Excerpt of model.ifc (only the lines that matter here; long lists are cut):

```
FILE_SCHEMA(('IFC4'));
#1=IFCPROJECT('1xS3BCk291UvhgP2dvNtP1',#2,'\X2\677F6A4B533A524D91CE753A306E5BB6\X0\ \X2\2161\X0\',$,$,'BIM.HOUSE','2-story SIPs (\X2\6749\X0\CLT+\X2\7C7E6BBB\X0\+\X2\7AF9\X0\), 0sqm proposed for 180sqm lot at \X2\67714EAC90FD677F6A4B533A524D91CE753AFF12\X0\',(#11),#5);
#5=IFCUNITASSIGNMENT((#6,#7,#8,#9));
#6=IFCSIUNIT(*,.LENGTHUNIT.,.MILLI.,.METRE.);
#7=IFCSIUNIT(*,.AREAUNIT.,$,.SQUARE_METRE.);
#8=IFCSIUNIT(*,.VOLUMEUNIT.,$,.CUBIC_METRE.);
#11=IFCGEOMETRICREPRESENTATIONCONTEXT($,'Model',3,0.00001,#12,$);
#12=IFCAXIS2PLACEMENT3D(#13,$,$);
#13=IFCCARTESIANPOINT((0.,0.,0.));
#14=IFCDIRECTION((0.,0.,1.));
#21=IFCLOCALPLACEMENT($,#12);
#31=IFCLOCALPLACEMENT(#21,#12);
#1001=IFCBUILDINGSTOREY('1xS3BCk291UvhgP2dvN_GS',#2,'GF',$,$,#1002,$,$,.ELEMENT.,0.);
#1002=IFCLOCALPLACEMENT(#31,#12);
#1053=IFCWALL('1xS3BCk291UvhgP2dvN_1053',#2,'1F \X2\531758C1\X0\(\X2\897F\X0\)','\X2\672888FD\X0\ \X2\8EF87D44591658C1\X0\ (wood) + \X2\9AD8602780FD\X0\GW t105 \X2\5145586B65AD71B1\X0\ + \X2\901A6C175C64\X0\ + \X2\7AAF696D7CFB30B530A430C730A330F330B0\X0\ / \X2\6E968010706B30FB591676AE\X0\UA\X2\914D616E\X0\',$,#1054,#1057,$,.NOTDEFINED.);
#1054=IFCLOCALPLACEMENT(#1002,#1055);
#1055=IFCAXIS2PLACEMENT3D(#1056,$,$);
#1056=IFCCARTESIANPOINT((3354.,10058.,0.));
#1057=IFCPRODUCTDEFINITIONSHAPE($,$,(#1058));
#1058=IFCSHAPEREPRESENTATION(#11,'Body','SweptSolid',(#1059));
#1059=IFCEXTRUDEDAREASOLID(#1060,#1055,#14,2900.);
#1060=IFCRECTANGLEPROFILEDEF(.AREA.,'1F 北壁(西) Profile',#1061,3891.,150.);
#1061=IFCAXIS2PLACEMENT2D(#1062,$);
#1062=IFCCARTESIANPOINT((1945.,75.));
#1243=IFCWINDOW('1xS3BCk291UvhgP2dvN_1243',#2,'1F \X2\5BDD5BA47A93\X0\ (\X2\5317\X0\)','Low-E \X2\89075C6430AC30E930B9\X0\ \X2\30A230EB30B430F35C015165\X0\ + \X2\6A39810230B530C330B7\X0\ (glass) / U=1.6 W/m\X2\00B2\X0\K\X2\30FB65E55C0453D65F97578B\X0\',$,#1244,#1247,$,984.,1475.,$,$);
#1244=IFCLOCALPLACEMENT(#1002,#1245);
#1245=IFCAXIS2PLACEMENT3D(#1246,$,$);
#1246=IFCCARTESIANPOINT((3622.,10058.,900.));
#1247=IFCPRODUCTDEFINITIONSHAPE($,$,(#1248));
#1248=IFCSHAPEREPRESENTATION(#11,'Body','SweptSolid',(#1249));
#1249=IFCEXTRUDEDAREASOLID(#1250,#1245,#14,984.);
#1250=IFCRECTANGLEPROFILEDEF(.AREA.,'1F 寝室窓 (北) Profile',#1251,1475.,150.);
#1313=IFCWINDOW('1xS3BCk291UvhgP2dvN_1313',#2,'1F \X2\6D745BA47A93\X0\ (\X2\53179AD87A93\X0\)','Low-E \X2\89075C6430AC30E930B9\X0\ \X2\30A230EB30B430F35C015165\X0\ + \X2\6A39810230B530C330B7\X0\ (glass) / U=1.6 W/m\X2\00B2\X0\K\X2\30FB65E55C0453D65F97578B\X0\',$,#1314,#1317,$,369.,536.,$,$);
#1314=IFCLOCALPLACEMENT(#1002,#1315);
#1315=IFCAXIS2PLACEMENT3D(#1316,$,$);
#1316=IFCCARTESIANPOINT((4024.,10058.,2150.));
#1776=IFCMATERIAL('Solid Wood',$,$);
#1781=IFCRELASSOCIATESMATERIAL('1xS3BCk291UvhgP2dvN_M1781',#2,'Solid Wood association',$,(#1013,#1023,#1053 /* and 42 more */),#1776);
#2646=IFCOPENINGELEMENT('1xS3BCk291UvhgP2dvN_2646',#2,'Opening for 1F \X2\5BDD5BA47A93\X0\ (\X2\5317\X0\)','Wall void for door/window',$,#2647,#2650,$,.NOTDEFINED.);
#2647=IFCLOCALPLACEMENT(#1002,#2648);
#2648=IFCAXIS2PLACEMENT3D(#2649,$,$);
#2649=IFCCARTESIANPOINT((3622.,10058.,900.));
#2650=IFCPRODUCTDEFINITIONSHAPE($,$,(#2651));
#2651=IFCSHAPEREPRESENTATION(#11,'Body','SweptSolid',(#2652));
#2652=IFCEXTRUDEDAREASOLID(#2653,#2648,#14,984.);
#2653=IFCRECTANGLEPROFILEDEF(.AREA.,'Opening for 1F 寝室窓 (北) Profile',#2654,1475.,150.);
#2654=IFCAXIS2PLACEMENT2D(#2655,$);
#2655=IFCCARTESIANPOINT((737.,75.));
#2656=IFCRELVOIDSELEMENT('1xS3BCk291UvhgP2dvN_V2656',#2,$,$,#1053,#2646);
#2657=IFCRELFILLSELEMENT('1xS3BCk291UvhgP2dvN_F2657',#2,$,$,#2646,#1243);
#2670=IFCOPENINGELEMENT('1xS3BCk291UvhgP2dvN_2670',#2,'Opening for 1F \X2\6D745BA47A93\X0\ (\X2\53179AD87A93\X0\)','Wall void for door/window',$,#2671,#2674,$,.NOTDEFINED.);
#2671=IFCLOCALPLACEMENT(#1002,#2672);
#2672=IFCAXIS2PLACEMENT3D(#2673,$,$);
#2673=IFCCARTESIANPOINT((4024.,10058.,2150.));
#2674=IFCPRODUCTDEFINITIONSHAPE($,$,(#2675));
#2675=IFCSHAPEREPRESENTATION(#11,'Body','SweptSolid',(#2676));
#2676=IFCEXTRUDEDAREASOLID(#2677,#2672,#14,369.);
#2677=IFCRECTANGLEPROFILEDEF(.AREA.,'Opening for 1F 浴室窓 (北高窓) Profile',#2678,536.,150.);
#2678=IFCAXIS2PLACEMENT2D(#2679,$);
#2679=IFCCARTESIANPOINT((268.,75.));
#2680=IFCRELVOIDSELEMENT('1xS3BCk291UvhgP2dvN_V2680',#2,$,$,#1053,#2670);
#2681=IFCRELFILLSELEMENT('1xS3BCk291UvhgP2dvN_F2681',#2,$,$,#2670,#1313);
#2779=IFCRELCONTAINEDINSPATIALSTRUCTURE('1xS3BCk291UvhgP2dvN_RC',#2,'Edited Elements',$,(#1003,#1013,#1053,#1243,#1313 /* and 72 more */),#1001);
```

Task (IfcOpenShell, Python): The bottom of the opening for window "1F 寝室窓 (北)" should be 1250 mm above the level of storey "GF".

```python
import numpy as np
import ifcopenshell
import ifcopenshell.api.geometry
import ifcopenshell.geom
import ifcopenshell.util.element
import ifcopenshell.util.placement
import ifcopenshell.util.shape
import ifcopenshell.util.unit

model = ifcopenshell.open("model.ifc")
unit_scale = ifcopenshell.util.unit.calculate_unit_scale(model)

window = model.by_guid("1xS3BCk291UvhgP2dvN_1243")
opening = window.FillsVoids[0].RelatingOpeningElement
storey = ifcopenshell.util.element.get_container(window, ifc_class="IfcBuildingStorey")
level = ifcopenshell.util.placement.get_local_placement(storey.ObjectPlacement)[2, 3]

# The opening's origin need not be at the sill, so measure its lowest point.
shape = ifcopenshell.geom.create_shape(ifcopenshell.geom.settings(), opening)
bottom = ifcopenshell.util.shape.get_shape_bottom_elevation(shape, shape.geometry) / unit_scale
dz = level + 1250.0 - bottom

shift = np.array([0.0, 0.0, dz])
# The window is not placed relative to its opening, so move both.
for product in (opening, window):
    matrix = ifcopenshell.util.placement.get_local_placement(product.ObjectPlacement)
    matrix[:3, 3] += shift
    ifcopenshell.api.geometry.edit_object_placement(model, product=product, matrix=matrix, is_si=False)

print(f"moved by {dz * unit_scale:+.3f} m")

model.write("model_updated.ifc")
```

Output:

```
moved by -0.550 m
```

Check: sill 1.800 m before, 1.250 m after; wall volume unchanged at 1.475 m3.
